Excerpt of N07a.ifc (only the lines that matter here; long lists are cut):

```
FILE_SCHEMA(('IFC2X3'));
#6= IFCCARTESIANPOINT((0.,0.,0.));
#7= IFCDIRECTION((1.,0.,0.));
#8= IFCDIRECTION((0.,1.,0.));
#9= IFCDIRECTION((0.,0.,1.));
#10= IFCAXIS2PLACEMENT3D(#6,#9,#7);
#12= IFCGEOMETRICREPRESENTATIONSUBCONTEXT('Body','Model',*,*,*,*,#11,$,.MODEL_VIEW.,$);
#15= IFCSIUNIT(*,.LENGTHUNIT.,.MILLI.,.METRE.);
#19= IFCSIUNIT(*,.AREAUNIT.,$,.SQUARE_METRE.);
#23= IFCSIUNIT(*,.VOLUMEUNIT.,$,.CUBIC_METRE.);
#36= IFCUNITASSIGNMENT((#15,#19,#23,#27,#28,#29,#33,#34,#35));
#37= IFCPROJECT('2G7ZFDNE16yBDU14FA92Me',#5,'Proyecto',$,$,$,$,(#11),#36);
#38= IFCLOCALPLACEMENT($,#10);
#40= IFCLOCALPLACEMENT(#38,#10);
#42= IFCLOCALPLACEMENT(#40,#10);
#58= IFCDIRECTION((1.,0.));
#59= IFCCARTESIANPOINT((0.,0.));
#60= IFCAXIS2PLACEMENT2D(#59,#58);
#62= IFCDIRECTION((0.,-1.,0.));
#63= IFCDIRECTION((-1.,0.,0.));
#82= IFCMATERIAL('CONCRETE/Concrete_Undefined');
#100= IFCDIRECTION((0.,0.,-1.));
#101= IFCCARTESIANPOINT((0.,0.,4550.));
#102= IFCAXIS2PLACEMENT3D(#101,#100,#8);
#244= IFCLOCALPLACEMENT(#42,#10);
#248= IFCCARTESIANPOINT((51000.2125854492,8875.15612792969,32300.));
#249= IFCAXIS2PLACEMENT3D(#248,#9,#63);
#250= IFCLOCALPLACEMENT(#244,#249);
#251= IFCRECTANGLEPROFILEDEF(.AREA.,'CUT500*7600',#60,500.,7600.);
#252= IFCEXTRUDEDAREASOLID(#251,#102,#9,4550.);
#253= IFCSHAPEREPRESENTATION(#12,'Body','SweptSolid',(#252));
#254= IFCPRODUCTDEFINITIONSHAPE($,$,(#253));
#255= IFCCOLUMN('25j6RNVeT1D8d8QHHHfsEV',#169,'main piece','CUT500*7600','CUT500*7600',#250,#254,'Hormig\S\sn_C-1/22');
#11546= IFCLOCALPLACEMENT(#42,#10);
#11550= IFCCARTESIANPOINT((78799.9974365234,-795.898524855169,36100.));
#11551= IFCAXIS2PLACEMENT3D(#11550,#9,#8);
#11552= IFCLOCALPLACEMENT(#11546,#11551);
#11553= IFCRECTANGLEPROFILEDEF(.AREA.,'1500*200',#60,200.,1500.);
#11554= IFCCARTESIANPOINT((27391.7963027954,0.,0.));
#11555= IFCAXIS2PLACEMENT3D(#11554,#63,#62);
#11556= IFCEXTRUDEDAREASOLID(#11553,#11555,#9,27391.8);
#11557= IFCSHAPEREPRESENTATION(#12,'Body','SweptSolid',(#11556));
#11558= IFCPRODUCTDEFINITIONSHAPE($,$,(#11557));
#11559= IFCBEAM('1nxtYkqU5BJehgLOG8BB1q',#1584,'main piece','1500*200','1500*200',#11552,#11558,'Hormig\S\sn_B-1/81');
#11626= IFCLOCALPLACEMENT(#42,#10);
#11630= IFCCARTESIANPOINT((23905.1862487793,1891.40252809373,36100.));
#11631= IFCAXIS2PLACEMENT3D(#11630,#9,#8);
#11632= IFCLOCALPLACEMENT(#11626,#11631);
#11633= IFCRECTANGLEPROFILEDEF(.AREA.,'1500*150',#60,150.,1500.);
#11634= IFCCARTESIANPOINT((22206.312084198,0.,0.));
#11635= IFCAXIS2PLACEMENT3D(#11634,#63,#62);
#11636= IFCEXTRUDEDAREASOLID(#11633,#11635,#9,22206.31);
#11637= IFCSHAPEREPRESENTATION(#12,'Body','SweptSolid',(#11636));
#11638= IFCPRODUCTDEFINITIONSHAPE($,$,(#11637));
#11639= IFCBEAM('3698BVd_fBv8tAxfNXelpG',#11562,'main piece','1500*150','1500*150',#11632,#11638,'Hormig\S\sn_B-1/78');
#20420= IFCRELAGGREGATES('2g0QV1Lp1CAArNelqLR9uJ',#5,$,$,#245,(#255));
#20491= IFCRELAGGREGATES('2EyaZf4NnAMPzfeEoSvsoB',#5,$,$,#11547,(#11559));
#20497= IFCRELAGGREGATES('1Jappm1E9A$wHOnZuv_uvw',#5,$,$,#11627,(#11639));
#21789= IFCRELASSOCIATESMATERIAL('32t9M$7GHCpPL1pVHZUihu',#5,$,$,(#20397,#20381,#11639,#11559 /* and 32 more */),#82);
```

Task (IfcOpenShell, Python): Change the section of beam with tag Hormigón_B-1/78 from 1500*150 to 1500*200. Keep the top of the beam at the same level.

```python
import ifcopenshell
import ifcopenshell.util.element
import ifcopenshell.util.representation

model = ifcopenshell.open("N07a.ifc")

member = model.by_guid("3698BVd_fBv8tAxfNXelpG")
source = next(p for p in model.by_type("IfcRectangleProfileDef") if p.ProfileName == "1500*200")

body = ifcopenshell.util.representation.get_representation(member, "Model", "Body")
solid = body.Items[0]
old_profile = solid.SweptArea

# Copy the section's sizes but keep this member's own profile position.
profile = ifcopenshell.util.element.copy(model, source)
# Profiles are centred, so shift by half the change in depth to hold the top.
shift = (old_profile.YDim - profile.YDim) / 2
x, y = old_profile.Position.Location.Coordinates
up = (0.0, 1.0)  # upwards, in the solid's own plane
location = model.createIfcCartesianPoint((x + up[0] * shift, y + up[1] * shift))
profile.Position = model.createIfcAxis2Placement2D(location, old_profile.Position.RefDirection)
solid.SweptArea = profile
if not model.get_total_inverses(old_profile):
    ifcopenshell.util.element.remove_deep2(model, old_profile)
member.Description = member.Description.replace("1500*150", "1500*200")
member.ObjectType = member.ObjectType.replace("1500*150", "1500*200")

print(solid.SweptArea)

model.write("N07a_rev.ifc")
```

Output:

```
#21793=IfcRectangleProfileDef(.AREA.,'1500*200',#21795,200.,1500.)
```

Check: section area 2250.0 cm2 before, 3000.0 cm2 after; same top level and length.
